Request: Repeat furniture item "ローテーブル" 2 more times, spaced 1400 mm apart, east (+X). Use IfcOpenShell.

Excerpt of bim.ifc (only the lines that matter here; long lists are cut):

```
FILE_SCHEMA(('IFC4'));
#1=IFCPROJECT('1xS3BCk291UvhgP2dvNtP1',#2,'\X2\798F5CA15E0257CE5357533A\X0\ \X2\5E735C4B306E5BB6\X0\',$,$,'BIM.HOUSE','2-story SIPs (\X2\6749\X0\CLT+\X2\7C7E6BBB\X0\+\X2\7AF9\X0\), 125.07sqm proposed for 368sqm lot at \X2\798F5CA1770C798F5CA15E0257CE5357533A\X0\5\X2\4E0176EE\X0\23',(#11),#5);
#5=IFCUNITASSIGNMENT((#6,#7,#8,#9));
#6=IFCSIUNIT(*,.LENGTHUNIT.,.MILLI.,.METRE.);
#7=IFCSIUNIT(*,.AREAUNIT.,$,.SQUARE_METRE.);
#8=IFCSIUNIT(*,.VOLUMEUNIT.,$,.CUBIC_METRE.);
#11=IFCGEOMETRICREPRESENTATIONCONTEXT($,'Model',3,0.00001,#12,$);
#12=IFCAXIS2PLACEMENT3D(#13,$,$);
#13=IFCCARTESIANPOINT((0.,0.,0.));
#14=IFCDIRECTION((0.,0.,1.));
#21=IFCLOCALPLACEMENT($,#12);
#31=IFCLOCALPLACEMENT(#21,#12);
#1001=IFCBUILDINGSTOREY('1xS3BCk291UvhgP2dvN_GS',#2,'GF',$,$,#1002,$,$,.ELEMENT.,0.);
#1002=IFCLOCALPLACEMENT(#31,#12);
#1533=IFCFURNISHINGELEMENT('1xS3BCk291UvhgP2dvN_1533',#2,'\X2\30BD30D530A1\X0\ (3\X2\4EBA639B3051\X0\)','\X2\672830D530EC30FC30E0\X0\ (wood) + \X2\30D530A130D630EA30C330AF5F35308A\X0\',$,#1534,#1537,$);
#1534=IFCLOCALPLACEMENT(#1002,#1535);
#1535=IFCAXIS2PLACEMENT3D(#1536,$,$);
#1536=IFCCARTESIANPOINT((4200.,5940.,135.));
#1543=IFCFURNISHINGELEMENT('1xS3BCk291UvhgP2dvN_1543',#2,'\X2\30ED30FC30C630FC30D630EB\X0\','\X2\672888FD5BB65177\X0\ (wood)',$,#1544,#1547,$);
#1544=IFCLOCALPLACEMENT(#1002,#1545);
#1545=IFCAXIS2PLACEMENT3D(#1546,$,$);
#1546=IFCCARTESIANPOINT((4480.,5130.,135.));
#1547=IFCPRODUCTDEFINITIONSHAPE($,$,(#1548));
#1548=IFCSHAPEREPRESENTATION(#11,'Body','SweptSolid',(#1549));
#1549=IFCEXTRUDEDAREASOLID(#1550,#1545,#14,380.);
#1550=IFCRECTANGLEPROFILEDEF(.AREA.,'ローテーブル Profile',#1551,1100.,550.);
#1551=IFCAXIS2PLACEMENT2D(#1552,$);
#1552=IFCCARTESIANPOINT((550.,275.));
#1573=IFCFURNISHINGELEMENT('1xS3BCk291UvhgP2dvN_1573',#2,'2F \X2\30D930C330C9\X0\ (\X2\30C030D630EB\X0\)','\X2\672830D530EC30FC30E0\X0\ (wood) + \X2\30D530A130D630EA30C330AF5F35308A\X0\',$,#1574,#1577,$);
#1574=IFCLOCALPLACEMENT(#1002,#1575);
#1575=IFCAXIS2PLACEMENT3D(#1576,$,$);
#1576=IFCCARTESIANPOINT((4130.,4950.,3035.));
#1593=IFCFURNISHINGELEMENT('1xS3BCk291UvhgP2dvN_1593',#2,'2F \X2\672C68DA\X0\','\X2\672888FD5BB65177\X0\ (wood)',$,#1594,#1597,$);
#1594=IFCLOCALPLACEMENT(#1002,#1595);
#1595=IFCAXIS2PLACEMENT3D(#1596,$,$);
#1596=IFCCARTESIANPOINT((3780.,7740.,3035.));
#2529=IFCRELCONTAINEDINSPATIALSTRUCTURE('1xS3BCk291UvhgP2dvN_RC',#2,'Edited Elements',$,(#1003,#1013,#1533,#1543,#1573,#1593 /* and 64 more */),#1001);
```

```python
import numpy as np
import ifcopenshell
import ifcopenshell.api.geometry
import ifcopenshell.api.root
import ifcopenshell.util.element
import ifcopenshell.util.placement

model = ifcopenshell.open("bim.ifc")


def reuse_history(source, copy):
    """copy_class also copies each property set's owner history, people and application; keep the originals."""
    for rel in copy.IsDefinedBy:
        if rel.is_a("IfcRelDefinesByProperties") and (history := rel.RelatingPropertyDefinition.OwnerHistory):
            rel.RelatingPropertyDefinition.OwnerHistory = source.OwnerHistory
            ifcopenshell.util.element.remove_deep2(model, history)


source = model.by_guid("1xS3BCk291UvhgP2dvN_1543")
base = ifcopenshell.util.placement.get_local_placement(source.ObjectPlacement)
step = np.array([1.0, 0.0, 0.0]) * 1400.0

for i in range(1, 3):
    copy = ifcopenshell.api.root.copy_class(model, product=source)
    copy.Representation = ifcopenshell.util.element.copy_deep(
        model, source.Representation, exclude=["IfcGeometricRepresentationContext", "IfcRepresentationMap"]
    )
    reuse_history(source, copy)
    matrix = base.copy()
    matrix[:3, 3] += i * step
    print("added at", matrix[:3, 3].round(3) + 0.0)
    ifcopenshell.api.geometry.edit_object_placement(model, product=copy, matrix=matrix, is_si=False)

model.write("bim_edited.ifc")
```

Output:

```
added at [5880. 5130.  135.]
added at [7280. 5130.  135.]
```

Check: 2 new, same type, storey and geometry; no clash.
